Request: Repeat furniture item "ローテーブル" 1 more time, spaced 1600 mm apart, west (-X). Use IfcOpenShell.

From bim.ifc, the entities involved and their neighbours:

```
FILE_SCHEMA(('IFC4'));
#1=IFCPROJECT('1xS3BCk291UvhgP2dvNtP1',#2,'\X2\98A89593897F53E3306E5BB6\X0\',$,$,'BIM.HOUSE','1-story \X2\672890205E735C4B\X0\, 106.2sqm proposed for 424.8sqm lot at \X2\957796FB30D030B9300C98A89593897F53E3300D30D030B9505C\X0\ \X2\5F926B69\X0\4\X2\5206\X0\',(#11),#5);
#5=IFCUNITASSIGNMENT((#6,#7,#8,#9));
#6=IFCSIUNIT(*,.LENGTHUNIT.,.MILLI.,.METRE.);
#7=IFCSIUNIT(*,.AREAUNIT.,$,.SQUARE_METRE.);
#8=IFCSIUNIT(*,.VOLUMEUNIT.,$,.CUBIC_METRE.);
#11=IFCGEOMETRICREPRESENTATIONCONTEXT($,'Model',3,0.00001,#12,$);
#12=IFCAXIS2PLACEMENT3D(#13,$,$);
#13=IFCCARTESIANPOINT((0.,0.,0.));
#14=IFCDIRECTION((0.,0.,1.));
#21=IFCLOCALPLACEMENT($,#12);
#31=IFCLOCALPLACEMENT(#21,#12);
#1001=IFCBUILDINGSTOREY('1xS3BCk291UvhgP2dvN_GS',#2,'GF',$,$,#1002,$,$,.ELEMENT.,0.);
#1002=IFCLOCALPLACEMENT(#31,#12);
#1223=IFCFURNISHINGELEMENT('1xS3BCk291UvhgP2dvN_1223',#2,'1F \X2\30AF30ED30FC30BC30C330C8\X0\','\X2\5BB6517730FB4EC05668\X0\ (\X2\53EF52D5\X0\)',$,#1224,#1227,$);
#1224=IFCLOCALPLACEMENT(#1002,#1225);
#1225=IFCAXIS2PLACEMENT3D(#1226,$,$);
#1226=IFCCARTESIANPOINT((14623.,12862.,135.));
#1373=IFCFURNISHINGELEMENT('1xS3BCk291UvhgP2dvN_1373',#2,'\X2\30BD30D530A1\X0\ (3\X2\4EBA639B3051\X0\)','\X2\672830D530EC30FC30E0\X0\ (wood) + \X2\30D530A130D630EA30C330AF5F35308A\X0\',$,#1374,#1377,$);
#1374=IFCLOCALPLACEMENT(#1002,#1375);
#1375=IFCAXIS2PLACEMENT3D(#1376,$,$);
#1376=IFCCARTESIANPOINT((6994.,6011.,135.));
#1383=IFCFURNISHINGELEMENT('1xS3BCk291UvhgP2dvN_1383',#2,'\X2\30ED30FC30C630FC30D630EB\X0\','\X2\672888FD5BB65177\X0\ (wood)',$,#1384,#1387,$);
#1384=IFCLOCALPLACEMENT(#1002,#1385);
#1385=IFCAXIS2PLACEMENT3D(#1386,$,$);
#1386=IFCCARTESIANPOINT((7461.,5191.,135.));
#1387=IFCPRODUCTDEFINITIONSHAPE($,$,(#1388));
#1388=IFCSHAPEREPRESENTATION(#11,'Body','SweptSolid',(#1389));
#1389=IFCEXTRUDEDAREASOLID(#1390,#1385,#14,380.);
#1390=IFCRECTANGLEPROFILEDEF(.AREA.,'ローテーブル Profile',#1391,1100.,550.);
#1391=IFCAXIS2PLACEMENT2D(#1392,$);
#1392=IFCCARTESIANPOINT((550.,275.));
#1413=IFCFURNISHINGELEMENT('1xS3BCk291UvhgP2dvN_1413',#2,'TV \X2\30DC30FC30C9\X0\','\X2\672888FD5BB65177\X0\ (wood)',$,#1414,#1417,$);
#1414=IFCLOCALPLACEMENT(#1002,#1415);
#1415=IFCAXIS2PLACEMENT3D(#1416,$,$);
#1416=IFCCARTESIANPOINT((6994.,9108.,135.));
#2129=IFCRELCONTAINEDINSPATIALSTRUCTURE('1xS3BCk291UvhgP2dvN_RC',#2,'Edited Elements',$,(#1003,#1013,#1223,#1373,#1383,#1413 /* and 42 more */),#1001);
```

```python
import numpy as np
import ifcopenshell
import ifcopenshell.api.geometry
import ifcopenshell.api.root
import ifcopenshell.util.element
import ifcopenshell.util.placement

model = ifcopenshell.open("bim.ifc")


def reuse_history(source, copy):
    """copy_class also copies each property set's owner history, people and application; keep the originals."""
    for rel in copy.IsDefinedBy:
        if rel.is_a("IfcRelDefinesByProperties") and (history := rel.RelatingPropertyDefinition.OwnerHistory):
            rel.RelatingPropertyDefinition.OwnerHistory = source.OwnerHistory
            ifcopenshell.util.element.remove_deep2(model, history)


source = model.by_guid("1xS3BCk291UvhgP2dvN_1383")
base = ifcopenshell.util.placement.get_local_placement(source.ObjectPlacement)
step = np.array([-1.0, 0.0, 0.0]) * 1600.0

for i in range(1, 2):
    copy = ifcopenshell.api.root.copy_class(model, product=source)
    copy.Representation = ifcopenshell.util.element.copy_deep(
        model, source.Representation, exclude=["IfcGeometricRepresentationContext", "IfcRepresentationMap"]
    )
    reuse_history(source, copy)
    matrix = base.copy()
    matrix[:3, 3] += i * step
    print("added at", matrix[:3, 3].round(3) + 0.0)
    ifcopenshell.api.geometry.edit_object_placement(model, product=copy, matrix=matrix, is_si=False)

model.write("bim-out.ifc")
```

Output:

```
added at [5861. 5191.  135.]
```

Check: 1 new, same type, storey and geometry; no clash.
